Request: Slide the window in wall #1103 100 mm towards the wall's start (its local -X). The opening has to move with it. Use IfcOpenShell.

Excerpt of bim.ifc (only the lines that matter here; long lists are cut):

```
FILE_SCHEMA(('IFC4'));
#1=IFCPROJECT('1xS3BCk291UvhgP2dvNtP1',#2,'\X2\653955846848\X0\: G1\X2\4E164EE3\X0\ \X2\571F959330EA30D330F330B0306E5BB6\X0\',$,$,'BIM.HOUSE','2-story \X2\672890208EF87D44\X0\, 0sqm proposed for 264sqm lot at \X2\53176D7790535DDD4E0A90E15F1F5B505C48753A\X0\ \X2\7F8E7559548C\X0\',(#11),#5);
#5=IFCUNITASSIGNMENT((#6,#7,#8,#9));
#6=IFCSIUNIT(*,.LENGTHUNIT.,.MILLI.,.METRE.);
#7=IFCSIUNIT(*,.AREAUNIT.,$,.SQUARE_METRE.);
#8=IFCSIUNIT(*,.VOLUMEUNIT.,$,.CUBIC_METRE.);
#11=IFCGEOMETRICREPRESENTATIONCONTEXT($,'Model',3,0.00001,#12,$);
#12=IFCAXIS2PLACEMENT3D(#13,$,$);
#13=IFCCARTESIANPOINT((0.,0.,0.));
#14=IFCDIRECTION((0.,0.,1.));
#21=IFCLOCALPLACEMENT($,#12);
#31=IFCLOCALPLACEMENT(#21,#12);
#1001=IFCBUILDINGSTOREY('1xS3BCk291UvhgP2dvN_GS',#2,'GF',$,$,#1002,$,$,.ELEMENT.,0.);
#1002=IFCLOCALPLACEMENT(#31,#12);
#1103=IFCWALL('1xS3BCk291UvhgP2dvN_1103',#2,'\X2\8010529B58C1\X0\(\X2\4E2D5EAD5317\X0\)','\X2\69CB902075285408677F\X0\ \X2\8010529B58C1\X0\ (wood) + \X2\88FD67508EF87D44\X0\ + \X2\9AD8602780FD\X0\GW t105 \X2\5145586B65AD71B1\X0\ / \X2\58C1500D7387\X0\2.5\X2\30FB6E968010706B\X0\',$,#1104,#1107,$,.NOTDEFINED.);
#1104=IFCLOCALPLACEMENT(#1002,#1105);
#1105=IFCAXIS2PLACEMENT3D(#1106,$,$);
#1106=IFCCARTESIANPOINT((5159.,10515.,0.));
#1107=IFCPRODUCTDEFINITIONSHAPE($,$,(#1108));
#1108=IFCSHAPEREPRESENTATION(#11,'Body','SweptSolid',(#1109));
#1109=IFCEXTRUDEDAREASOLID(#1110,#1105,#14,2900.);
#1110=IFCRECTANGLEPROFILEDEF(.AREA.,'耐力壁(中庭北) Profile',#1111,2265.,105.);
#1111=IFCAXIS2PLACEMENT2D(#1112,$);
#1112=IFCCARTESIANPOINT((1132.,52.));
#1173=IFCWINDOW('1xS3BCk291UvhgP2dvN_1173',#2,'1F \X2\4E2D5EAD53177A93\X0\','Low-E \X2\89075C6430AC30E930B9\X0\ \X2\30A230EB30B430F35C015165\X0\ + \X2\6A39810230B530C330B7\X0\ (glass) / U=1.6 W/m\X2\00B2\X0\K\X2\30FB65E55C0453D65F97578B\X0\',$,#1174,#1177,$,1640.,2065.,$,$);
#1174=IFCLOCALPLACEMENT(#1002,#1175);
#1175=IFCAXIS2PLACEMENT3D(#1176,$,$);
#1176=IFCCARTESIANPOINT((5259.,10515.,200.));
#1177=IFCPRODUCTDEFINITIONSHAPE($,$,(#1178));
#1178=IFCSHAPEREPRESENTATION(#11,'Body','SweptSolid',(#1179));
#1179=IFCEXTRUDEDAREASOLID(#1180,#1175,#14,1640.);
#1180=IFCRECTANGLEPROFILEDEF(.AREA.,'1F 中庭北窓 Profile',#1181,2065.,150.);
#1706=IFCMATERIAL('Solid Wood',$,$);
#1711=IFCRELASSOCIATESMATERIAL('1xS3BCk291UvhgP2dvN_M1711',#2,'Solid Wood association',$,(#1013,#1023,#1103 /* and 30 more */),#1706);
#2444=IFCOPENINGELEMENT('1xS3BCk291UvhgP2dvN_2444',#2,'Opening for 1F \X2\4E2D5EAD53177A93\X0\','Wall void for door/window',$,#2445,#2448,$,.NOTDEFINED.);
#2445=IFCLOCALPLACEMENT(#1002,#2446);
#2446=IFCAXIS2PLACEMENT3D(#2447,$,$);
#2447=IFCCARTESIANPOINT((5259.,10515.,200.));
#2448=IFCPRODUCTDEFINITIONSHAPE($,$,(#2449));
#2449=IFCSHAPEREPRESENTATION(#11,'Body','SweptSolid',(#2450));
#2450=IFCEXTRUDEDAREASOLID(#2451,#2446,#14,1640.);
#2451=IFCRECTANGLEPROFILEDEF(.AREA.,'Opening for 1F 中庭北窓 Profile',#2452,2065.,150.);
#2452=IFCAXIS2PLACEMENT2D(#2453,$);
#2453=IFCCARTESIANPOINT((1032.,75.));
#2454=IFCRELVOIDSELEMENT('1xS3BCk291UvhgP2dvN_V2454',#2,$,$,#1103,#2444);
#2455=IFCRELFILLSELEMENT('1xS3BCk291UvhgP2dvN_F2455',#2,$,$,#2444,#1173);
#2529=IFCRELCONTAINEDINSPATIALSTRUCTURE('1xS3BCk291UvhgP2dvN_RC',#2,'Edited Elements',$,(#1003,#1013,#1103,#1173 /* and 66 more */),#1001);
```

```python
import ifcopenshell
import ifcopenshell.api.geometry
import ifcopenshell.util.placement
import ifcopenshell.util.unit

model = ifcopenshell.open("bim.ifc")
unit_scale = ifcopenshell.util.unit.calculate_unit_scale(model)

window = model.by_guid("1xS3BCk291UvhgP2dvN_1173")
opening = window.FillsVoids[0].RelatingOpeningElement
wall = opening.VoidsElements[0].RelatingBuildingElement

wall_matrix = ifcopenshell.util.placement.get_local_placement(wall.ObjectPlacement)
shift = wall_matrix[:3, 0] * -0.1 / unit_scale
before = ifcopenshell.util.placement.get_local_placement(window.ObjectPlacement)[:3, 3].copy()

# The window is not placed relative to its opening, so move both.
for product in (opening, window):
    matrix = ifcopenshell.util.placement.get_local_placement(product.ObjectPlacement)
    matrix[:3, 3] += shift
    ifcopenshell.api.geometry.edit_object_placement(model, product=product, matrix=matrix, is_si=False)

after = ifcopenshell.util.placement.get_local_placement(window.ObjectPlacement)[:3, 3]
print("window moved by", (after - before).round(3) + 0.0)

model.write("bim_rev.ifc")
```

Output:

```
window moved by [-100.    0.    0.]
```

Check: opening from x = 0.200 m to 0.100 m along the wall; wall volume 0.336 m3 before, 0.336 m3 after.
